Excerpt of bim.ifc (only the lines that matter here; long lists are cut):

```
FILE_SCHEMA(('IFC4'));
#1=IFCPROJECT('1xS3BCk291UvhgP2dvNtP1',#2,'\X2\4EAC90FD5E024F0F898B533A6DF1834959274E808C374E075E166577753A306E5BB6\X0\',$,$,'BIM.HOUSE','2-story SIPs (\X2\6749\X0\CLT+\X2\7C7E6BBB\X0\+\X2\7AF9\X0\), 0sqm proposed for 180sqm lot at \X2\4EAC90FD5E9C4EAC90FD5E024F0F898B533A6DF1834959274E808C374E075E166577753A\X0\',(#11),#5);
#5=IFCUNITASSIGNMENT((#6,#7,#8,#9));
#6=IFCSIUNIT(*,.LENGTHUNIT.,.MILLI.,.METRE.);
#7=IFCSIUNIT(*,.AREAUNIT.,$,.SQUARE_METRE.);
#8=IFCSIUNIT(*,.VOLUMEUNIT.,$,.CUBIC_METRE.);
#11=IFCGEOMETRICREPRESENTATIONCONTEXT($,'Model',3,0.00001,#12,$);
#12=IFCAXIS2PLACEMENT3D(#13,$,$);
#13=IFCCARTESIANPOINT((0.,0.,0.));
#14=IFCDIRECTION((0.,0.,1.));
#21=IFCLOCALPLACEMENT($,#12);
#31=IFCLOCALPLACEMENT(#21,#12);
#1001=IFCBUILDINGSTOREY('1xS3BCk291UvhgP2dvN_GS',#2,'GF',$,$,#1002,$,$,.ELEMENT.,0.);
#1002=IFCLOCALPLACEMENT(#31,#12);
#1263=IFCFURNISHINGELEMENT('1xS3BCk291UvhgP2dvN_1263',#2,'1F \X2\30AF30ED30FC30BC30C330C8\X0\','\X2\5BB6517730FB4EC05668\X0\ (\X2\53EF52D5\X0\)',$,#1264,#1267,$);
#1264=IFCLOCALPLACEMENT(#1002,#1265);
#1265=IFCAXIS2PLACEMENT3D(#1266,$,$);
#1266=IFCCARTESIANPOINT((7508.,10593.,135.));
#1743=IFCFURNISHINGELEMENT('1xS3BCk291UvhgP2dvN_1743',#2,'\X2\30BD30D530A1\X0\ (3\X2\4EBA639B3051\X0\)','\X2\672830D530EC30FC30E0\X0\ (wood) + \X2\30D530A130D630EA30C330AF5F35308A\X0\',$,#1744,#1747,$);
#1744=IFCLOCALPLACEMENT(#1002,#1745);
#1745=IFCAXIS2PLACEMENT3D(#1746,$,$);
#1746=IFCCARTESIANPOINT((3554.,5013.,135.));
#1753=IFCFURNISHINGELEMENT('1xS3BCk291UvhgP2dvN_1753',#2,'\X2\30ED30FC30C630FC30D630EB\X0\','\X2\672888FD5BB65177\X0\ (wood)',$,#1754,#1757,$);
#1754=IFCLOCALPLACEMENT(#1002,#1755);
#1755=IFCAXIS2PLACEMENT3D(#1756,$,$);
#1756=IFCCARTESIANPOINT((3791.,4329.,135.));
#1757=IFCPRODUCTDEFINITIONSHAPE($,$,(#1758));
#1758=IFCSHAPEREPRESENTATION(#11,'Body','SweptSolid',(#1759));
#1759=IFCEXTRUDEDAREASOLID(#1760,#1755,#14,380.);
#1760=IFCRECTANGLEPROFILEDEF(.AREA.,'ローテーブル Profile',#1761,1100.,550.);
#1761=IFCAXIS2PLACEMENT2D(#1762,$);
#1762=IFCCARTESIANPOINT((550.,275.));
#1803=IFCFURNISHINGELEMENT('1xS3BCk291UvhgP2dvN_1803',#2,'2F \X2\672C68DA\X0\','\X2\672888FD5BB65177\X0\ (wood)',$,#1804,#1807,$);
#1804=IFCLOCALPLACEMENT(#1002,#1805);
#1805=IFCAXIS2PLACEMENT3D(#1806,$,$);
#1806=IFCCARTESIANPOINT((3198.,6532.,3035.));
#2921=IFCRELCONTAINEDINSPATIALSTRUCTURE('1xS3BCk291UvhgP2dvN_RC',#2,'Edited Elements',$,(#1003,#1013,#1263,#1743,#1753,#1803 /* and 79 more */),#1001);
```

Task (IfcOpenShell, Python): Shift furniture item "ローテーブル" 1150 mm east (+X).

```python
import ifcopenshell
import ifcopenshell.api.geometry
import ifcopenshell.util.placement
import ifcopenshell.util.unit

model = ifcopenshell.open("bim.ifc")
unit_scale = ifcopenshell.util.unit.calculate_unit_scale(model)

item = model.by_guid("1xS3BCk291UvhgP2dvN_1753")
matrix = ifcopenshell.util.placement.get_local_placement(item.ObjectPlacement)
matrix[0, 3] += 1.15 / unit_scale
ifcopenshell.api.geometry.edit_object_placement(model, product=item, matrix=matrix, is_si=False)

print(ifcopenshell.util.placement.get_local_placement(item.ObjectPlacement).round(3) + 0.0)

model.write("bim_edited.ifc")
```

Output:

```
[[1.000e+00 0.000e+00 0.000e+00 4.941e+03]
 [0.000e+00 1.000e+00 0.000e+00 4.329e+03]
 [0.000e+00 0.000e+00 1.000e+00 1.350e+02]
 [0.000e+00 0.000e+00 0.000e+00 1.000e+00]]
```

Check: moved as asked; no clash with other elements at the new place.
